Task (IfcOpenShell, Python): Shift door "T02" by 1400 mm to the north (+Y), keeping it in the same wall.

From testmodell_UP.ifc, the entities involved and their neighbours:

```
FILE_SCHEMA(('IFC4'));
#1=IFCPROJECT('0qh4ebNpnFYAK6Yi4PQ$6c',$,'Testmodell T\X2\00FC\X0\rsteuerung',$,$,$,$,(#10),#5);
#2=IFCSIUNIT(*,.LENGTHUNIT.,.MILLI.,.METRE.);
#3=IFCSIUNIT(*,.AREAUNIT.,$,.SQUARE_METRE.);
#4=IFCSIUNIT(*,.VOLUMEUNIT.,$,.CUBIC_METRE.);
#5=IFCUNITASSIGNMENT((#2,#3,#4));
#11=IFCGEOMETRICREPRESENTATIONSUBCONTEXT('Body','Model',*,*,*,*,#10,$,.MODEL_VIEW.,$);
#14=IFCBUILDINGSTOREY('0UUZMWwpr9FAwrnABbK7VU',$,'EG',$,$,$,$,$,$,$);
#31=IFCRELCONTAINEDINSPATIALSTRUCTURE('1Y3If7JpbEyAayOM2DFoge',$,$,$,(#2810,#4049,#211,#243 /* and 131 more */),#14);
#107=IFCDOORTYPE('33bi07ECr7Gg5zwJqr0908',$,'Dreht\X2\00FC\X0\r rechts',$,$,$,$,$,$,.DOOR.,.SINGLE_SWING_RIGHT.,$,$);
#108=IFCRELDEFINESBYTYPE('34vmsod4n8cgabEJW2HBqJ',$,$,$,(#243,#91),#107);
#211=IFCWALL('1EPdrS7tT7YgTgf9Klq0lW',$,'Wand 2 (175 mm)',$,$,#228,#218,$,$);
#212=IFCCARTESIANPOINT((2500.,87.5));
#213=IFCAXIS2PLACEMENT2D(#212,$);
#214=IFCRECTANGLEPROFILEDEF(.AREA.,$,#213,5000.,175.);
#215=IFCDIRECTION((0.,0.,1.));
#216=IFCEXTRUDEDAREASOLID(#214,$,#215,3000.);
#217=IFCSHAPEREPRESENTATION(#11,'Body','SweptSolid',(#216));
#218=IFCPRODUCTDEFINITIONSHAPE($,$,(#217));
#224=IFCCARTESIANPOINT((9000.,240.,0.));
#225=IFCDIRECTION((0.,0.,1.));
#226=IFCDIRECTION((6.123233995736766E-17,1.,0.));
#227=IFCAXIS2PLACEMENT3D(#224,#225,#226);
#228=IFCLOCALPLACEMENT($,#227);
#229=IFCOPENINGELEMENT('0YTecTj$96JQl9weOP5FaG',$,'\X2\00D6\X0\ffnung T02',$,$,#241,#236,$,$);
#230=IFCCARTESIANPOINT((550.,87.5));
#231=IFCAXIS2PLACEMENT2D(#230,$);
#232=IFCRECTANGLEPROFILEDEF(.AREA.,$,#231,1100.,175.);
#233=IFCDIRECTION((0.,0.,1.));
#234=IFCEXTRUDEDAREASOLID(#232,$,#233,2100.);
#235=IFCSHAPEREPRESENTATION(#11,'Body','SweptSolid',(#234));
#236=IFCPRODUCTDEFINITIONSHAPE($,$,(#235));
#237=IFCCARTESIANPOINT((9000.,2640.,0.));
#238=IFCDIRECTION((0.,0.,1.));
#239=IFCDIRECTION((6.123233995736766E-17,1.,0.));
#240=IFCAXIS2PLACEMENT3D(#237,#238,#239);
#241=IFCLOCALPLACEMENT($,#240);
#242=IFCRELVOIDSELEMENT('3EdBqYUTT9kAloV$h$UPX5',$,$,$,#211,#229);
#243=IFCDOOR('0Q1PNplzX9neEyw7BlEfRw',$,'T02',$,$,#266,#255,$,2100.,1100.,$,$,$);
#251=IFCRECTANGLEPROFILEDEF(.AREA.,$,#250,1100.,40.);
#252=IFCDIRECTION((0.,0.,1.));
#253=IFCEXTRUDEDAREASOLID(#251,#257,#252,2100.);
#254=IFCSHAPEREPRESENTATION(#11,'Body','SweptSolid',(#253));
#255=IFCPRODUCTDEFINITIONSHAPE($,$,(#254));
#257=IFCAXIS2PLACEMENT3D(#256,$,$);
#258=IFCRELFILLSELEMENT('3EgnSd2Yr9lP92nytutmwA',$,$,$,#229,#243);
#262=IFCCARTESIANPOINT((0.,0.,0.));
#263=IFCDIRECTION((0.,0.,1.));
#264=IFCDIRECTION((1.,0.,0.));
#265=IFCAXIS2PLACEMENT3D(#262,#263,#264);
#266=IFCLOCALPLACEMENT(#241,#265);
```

```python
import ifcopenshell
import ifcopenshell.api.geometry
import ifcopenshell.util.placement

model = ifcopenshell.open("testmodell_UP.ifc")

door = model.by_guid("0Q1PNplzX9neEyw7BlEfRw")
opening = door.FillsVoids[0].RelatingOpeningElement
wall = opening.VoidsElements[0].RelatingBuildingElement

wall_matrix = ifcopenshell.util.placement.get_local_placement(wall.ObjectPlacement)
shift = wall_matrix[:3, 0] * 1400.0
before = ifcopenshell.util.placement.get_local_placement(door.ObjectPlacement)[:3, 3].copy()

# The door is placed relative to its opening, so it follows when the opening moves.
matrix = ifcopenshell.util.placement.get_local_placement(opening.ObjectPlacement)
matrix[:3, 3] += shift
ifcopenshell.api.geometry.edit_object_placement(
    model, product=opening, matrix=matrix, is_si=False, should_transform_children=True
)

after = ifcopenshell.util.placement.get_local_placement(door.ObjectPlacement)[:3, 3]
print("door moved by", (after - before).round(3) + 0.0)

model.write("testmodell_UP-out.ifc")
```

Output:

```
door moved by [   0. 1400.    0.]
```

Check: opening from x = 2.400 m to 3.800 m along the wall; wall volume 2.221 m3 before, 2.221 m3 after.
